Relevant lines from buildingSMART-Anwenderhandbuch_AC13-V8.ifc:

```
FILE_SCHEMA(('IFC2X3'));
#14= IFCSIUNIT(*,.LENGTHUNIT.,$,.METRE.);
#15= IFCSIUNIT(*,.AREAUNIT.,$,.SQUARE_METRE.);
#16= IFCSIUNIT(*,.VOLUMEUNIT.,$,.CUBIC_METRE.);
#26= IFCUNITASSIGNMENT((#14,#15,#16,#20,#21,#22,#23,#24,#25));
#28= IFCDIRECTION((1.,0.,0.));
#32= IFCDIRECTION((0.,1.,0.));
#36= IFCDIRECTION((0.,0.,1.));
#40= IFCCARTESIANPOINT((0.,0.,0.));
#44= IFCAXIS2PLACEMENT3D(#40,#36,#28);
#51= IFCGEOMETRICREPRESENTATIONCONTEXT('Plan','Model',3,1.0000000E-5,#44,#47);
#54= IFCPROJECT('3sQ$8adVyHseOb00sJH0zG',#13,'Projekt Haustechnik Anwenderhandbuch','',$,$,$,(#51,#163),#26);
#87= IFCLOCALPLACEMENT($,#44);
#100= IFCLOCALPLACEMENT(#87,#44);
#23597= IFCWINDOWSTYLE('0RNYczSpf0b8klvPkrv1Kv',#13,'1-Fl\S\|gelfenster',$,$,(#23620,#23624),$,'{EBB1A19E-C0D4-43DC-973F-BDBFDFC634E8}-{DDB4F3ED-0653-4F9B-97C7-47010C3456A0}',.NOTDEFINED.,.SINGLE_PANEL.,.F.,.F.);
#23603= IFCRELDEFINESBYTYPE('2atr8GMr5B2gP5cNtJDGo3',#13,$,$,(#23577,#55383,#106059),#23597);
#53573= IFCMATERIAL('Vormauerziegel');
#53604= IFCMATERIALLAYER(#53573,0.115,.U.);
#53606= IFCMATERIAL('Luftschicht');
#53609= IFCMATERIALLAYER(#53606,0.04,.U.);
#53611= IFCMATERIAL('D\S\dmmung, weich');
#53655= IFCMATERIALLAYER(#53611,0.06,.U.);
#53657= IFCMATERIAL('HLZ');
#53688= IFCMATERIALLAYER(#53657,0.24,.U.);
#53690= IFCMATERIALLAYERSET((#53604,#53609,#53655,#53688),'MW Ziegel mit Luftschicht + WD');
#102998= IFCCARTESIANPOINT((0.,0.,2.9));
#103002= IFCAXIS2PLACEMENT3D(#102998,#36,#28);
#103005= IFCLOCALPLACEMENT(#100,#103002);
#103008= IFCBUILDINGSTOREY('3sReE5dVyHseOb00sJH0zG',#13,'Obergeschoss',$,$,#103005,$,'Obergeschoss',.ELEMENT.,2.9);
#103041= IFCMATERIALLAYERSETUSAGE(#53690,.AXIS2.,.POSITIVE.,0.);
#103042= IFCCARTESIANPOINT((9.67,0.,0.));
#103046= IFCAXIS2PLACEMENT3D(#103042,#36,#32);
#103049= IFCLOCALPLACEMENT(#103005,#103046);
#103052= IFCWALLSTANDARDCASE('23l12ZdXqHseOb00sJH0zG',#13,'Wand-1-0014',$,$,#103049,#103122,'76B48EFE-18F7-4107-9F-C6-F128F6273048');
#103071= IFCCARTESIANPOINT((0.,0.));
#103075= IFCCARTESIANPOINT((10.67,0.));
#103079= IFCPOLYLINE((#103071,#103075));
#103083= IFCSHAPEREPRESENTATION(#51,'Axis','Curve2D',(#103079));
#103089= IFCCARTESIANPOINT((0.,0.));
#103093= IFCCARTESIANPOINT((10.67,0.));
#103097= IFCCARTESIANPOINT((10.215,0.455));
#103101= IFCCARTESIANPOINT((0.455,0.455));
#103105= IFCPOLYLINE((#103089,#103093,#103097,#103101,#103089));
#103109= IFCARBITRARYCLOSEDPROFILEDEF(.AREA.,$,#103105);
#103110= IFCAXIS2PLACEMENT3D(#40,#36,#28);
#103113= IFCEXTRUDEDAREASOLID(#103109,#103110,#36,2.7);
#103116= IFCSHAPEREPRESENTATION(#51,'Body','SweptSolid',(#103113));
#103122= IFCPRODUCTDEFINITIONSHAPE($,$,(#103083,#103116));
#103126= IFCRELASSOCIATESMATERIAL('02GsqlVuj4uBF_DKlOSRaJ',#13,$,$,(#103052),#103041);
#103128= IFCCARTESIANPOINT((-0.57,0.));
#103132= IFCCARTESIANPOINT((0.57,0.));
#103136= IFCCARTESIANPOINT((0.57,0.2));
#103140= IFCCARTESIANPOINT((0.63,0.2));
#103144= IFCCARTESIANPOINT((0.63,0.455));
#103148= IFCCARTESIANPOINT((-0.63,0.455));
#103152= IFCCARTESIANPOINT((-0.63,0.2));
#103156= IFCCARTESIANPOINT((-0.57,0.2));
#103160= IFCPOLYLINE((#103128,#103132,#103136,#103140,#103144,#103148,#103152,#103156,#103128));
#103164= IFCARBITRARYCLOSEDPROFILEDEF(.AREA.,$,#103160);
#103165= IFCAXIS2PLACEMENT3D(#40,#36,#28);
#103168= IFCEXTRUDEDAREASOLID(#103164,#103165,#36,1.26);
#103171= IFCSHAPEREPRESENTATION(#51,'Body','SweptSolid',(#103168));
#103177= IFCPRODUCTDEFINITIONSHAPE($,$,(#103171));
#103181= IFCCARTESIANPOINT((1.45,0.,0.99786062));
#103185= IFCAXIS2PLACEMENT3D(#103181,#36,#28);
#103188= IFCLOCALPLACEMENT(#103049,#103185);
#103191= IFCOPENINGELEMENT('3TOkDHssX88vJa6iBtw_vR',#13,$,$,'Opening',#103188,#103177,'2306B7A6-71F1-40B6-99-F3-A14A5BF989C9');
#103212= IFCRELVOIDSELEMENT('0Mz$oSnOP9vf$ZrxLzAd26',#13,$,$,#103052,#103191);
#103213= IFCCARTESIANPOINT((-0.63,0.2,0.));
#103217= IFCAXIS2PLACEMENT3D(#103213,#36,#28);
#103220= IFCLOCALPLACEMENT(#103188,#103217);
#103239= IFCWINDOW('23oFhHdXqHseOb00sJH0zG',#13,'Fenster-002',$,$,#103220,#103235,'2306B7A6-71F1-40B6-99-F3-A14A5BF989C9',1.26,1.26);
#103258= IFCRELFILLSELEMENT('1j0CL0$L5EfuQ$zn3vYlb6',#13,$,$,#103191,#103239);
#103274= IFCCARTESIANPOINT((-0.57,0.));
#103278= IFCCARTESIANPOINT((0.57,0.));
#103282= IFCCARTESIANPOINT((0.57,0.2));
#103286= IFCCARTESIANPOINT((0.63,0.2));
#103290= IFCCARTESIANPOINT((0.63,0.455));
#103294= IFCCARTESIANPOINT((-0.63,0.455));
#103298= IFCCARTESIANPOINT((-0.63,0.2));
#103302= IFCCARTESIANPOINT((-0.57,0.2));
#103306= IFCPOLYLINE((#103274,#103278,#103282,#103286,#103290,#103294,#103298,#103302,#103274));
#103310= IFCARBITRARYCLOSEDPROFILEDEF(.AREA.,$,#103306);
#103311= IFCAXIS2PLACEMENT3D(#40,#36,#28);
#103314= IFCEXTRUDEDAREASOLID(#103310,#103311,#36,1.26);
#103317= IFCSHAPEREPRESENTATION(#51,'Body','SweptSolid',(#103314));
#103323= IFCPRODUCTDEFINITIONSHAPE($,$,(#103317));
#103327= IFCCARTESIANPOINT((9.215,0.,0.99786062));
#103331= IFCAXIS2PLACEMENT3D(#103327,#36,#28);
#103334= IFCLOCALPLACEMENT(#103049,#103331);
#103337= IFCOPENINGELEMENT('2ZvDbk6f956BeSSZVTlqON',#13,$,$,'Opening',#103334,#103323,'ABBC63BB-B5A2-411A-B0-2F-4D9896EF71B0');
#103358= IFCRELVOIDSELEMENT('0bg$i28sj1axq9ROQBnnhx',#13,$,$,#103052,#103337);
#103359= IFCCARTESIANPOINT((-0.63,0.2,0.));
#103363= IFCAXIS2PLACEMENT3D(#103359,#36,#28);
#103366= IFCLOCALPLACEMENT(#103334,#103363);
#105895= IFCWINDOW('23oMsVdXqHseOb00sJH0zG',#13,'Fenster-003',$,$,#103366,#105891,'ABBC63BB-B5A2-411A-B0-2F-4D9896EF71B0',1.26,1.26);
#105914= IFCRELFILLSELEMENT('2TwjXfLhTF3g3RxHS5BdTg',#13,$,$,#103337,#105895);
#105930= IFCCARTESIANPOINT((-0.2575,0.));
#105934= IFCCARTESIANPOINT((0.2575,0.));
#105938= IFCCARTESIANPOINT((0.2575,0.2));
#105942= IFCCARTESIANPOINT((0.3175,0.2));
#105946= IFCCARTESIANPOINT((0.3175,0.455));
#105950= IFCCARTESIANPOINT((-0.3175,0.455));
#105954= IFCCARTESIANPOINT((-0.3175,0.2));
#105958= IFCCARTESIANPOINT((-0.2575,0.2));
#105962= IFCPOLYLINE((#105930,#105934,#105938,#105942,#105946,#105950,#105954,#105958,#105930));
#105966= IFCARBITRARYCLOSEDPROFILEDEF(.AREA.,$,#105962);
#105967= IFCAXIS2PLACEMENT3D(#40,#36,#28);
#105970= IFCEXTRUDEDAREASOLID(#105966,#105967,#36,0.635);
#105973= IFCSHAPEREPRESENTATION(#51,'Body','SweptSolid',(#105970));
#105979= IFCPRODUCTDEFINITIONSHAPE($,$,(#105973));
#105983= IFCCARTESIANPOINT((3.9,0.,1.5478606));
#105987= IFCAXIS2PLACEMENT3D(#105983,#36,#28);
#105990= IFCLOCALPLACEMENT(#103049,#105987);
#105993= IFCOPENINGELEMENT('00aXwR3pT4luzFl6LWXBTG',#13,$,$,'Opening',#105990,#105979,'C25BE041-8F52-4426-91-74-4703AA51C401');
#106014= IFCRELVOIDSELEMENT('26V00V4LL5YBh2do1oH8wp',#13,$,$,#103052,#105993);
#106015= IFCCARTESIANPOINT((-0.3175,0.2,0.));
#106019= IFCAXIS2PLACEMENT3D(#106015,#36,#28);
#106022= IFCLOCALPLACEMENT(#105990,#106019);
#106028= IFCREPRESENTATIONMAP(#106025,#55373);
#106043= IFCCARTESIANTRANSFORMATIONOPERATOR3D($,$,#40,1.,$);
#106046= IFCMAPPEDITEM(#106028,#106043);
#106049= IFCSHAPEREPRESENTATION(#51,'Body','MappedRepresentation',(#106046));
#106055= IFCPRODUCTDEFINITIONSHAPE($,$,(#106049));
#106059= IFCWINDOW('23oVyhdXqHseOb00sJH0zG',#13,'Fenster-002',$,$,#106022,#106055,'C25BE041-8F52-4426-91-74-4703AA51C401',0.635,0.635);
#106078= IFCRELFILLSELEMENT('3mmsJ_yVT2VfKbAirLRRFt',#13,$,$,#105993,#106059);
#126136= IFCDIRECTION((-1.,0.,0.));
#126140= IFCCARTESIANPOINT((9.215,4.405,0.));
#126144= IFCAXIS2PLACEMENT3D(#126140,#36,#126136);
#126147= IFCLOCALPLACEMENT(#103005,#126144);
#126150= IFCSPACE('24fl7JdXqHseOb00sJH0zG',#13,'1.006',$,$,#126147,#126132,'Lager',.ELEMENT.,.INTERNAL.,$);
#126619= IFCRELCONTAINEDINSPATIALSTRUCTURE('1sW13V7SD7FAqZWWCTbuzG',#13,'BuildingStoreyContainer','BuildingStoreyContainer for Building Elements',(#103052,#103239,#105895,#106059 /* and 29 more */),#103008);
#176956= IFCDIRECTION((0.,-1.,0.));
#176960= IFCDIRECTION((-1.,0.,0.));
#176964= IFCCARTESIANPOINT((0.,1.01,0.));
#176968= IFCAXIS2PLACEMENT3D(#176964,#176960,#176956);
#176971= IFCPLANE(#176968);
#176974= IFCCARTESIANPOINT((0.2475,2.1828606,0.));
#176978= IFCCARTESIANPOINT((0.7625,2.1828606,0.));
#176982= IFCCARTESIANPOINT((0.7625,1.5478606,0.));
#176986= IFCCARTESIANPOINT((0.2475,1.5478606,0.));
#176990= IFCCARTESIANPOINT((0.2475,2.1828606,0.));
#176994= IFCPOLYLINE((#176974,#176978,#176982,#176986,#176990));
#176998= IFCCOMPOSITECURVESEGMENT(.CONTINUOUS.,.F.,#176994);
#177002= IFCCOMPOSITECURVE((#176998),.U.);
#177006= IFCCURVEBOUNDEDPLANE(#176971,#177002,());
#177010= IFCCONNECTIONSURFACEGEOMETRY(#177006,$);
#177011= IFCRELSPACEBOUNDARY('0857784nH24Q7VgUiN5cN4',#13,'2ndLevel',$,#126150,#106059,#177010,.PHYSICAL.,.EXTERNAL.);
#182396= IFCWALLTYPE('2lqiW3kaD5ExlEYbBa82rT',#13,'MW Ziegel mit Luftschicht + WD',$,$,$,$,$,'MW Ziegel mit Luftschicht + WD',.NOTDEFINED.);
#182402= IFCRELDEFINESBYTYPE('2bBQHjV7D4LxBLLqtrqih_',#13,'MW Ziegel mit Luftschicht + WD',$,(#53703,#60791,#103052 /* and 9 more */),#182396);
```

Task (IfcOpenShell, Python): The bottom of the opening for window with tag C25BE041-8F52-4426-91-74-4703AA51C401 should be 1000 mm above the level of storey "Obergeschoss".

```python
import numpy as np
import ifcopenshell
import ifcopenshell.api.geometry
import ifcopenshell.geom
import ifcopenshell.util.element
import ifcopenshell.util.placement
import ifcopenshell.util.shape
import ifcopenshell.util.unit

model = ifcopenshell.open("buildingSMART-Anwenderhandbuch_AC13-V8.ifc")
unit_scale = ifcopenshell.util.unit.calculate_unit_scale(model)

window = model.by_guid("23oVyhdXqHseOb00sJH0zG")
opening = window.FillsVoids[0].RelatingOpeningElement
storey = ifcopenshell.util.element.get_container(window, ifc_class="IfcBuildingStorey")
level = ifcopenshell.util.placement.get_local_placement(storey.ObjectPlacement)[2, 3]

# The opening's origin need not be at the sill, so measure its lowest point.
shape = ifcopenshell.geom.create_shape(ifcopenshell.geom.settings(), opening)
bottom = ifcopenshell.util.shape.get_shape_bottom_elevation(shape, shape.geometry) / unit_scale
dz = level + 1 / unit_scale - bottom

shift = np.array([0.0, 0.0, dz])
# The window is placed relative to its opening, so it follows when the opening moves.
matrix = ifcopenshell.util.placement.get_local_placement(opening.ObjectPlacement)
matrix[:3, 3] += shift
ifcopenshell.api.geometry.edit_object_placement(
    model, product=opening, matrix=matrix, is_si=False, should_transform_children=True
)

# Space boundary surfaces are stored in each space's coordinates; move them too.
for rel in window.ProvidesBoundaries:
    if not rel.ConnectionGeometry:
        continue
    surface = rel.ConnectionGeometry.SurfaceOnRelatingElement.BasisSurface
    space_matrix = ifcopenshell.util.placement.get_local_placement(rel.RelatingSpace.ObjectPlacement)
    point = np.array(surface.Position.Location.Coordinates) + space_matrix[:3, :3].T @ shift
    surface.Position = model.createIfcAxis2Placement3D(
        model.createIfcCartesianPoint(point.tolist()), surface.Position.Axis, surface.Position.RefDirection
    )

print(f"moved by {dz * unit_scale:+.3f} m")

model.write("buildingSMART-Anwenderhandbuch_AC13-V8_rev.ifc")
```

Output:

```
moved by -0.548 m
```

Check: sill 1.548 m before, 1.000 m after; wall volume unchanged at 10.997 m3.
